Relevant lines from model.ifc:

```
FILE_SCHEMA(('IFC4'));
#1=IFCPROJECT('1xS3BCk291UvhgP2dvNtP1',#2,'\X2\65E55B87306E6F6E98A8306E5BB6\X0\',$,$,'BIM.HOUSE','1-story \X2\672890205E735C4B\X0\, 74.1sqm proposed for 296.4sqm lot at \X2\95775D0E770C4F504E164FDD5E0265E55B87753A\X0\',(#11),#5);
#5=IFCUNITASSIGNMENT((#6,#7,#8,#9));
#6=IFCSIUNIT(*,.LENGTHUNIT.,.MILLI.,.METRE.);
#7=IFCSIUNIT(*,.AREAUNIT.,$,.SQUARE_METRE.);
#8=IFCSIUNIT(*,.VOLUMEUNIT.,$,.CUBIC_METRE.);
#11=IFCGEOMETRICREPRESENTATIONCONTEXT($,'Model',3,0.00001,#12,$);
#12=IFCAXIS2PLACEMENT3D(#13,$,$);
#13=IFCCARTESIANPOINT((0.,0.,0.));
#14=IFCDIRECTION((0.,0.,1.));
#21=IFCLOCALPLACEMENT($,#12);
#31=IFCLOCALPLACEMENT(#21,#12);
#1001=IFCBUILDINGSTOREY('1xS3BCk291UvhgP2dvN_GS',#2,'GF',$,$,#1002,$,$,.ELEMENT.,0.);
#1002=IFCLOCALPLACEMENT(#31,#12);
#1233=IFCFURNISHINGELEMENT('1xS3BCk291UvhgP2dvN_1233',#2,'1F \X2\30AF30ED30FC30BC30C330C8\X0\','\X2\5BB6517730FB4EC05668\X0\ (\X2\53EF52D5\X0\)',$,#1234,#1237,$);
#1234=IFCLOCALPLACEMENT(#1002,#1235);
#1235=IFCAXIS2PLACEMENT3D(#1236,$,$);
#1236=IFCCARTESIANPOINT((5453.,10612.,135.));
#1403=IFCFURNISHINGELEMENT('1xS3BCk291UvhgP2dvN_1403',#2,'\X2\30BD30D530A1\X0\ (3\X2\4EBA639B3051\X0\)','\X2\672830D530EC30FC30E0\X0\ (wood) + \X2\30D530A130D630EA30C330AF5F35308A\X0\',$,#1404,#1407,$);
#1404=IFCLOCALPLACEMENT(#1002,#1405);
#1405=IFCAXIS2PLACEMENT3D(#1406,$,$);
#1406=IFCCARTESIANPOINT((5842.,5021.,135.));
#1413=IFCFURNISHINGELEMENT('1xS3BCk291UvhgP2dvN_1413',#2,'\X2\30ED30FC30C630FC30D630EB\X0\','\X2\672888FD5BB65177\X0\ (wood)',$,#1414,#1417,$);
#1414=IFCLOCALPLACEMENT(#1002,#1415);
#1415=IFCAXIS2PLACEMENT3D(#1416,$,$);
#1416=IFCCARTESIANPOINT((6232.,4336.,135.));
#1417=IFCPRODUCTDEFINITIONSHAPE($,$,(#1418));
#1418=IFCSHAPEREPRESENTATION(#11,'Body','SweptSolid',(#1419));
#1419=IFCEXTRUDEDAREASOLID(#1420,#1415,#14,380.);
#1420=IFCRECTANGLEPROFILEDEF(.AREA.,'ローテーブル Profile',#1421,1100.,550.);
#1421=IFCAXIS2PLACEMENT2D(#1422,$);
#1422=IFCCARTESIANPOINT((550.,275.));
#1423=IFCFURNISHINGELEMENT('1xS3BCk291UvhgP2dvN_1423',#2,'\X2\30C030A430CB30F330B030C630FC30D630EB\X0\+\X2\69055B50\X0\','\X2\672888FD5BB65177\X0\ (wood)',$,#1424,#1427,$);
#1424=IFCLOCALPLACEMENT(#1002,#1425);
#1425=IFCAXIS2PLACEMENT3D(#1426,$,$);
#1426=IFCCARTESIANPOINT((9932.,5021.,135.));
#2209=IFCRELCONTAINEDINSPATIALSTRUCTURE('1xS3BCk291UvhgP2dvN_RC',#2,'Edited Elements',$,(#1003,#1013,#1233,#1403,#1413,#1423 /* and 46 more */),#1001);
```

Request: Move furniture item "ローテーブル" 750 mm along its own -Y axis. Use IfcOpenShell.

```python
import ifcopenshell
import ifcopenshell.api.geometry
import ifcopenshell.util.placement
import ifcopenshell.util.unit

model = ifcopenshell.open("model.ifc")
unit_scale = ifcopenshell.util.unit.calculate_unit_scale(model)

item = model.by_id(1413)
matrix = ifcopenshell.util.placement.get_local_placement(item.ObjectPlacement)
matrix[:3, 3] -= matrix[:3, 1] * 0.75 / unit_scale
ifcopenshell.api.geometry.edit_object_placement(model, product=item, matrix=matrix, is_si=False)

print(ifcopenshell.util.placement.get_local_placement(item.ObjectPlacement).round(3) + 0.0)

model.write("model_rev.ifc")
```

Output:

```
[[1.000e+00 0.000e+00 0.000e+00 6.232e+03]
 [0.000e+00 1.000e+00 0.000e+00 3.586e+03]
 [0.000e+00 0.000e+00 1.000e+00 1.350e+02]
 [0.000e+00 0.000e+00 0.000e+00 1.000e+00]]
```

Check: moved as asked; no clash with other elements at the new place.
